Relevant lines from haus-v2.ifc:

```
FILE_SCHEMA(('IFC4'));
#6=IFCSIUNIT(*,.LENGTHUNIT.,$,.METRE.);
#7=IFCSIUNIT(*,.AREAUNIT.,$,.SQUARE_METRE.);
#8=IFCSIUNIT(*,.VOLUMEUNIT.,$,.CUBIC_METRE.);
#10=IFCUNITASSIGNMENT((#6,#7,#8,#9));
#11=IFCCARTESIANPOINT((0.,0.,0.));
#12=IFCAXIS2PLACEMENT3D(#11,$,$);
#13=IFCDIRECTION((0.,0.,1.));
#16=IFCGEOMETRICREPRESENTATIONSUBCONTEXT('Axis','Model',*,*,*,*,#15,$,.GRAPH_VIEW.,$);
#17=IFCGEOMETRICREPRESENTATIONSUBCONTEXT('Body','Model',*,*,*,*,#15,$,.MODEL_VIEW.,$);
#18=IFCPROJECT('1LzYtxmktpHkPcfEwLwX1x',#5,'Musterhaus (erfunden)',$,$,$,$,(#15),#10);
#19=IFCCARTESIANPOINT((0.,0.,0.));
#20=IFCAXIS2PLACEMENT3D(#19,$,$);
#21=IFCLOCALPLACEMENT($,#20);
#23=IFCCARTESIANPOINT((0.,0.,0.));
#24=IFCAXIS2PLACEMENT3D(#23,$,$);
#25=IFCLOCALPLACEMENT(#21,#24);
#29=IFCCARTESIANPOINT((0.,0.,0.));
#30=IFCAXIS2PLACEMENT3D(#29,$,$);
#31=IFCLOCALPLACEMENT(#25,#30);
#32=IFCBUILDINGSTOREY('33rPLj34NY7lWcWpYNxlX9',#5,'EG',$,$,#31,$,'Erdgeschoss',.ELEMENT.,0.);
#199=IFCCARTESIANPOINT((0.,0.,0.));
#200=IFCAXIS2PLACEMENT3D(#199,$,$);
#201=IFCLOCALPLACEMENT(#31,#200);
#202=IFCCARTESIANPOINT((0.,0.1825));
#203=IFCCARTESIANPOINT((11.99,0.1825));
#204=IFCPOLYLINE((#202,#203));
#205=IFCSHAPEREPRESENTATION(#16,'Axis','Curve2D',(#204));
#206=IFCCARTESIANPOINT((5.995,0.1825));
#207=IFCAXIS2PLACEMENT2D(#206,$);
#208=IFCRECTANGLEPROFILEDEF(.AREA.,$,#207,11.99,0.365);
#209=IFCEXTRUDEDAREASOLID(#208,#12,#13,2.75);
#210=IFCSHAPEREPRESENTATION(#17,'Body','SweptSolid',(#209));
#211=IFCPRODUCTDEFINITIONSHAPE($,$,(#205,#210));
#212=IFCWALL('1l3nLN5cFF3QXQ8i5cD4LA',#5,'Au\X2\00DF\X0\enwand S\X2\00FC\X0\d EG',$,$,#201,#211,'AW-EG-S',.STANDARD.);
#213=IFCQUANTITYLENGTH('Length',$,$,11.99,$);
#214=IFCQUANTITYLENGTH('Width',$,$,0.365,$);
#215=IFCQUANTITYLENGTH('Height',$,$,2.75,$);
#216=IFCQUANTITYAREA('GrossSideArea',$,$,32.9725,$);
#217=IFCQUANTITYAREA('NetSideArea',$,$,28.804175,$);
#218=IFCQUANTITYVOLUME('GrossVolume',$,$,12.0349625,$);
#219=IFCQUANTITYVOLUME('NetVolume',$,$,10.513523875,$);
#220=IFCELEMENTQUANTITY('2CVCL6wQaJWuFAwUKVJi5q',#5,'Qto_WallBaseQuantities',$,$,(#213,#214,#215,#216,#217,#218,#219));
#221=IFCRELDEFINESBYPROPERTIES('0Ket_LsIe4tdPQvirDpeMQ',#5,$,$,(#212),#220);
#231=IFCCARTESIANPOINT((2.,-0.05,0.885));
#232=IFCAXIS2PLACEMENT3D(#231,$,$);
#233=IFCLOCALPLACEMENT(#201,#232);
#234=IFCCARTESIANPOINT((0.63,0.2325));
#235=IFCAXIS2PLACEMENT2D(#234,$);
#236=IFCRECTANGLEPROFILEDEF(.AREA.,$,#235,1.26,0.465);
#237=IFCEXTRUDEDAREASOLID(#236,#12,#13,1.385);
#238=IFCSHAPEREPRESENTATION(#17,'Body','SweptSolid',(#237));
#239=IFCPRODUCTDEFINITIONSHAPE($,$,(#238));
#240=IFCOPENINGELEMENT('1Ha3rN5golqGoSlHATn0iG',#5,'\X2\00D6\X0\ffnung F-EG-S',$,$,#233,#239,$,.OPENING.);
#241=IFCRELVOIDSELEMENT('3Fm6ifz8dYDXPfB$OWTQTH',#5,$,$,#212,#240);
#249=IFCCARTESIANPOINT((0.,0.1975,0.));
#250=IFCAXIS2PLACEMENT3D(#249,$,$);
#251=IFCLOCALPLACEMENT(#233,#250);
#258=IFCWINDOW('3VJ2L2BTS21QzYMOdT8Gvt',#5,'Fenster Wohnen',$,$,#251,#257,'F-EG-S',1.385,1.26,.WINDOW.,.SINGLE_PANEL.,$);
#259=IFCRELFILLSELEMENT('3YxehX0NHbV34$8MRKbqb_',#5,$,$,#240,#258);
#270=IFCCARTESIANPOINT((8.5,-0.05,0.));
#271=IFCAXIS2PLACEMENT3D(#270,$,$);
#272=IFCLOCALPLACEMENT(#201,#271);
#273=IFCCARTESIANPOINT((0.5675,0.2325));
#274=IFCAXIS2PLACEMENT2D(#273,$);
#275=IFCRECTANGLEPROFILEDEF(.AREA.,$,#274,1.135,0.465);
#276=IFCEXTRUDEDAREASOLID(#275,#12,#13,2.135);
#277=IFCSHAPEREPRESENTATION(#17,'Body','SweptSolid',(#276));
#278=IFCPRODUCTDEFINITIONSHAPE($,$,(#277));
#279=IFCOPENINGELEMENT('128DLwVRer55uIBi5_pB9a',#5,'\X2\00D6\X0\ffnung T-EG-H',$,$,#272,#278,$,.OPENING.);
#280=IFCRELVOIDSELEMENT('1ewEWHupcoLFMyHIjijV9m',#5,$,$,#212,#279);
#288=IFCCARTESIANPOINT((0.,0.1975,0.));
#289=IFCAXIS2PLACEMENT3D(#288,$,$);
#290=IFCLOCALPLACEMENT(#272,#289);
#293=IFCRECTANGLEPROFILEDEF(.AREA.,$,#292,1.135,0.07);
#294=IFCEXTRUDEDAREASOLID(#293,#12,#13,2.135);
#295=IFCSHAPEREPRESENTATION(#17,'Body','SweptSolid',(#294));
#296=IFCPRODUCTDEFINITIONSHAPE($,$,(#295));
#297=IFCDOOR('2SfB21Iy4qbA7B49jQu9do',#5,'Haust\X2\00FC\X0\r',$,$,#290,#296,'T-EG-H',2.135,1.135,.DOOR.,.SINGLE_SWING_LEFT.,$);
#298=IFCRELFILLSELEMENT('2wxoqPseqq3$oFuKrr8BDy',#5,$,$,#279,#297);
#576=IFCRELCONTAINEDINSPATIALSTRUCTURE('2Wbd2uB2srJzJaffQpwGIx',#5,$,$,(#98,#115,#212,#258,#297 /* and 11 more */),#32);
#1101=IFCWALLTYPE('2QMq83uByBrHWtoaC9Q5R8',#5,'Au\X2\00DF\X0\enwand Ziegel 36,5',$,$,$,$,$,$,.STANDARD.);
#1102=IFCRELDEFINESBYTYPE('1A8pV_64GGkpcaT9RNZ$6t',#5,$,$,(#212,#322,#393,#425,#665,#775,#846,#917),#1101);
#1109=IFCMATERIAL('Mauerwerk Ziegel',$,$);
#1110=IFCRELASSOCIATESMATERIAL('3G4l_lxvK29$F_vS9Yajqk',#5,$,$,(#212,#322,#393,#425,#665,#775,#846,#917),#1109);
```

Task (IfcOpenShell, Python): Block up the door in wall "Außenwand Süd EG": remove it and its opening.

```python
import ifcopenshell
import ifcopenshell.api.feature
import ifcopenshell.api.pset
import ifcopenshell.api.root
import ifcopenshell.geom
import ifcopenshell.util.element
import ifcopenshell.util.shape
import ifcopenshell.util.unit

model = ifcopenshell.open("haus-v2.ifc")
area_scale = ifcopenshell.util.unit.calculate_unit_scale(model, "AREAUNIT")
volume_scale = ifcopenshell.util.unit.calculate_unit_scale(model, "VOLUMEUNIT")
settings = ifcopenshell.geom.settings()


def volume(element):
    """Net volume in cubic metres, openings subtracted."""
    shape = ifcopenshell.geom.create_shape(settings, element)
    return ifcopenshell.util.shape.get_volume(shape.geometry)


door = model.by_guid("2SfB21Iy4qbA7B49jQu9do")
opening = door.FillsVoids[0].RelatingOpeningElement
wall = opening.VoidsElements[0].RelatingBuildingElement
before = volume(wall)

ifcopenshell.api.root.remove_product(model, product=door)
ifcopenshell.api.feature.remove_feature(model, feature=opening)

after = volume(wall)
thickness = 0.365  # wall thickness in metres

# Update the wall's stored quantities.
qto = model.by_id(ifcopenshell.util.element.get_pset(wall, "Qto_WallBaseQuantities", should_inherit=False)["id"])
ifcopenshell.api.pset.edit_qto(model, qto=qto, properties={
    "NetSideArea": after / thickness / area_scale,
    "NetVolume": after / volume_scale,
})

print(f"wall volume {before:.3f} -> {after:.3f} m3")

model.write("haus-v2_rev.ifc")
```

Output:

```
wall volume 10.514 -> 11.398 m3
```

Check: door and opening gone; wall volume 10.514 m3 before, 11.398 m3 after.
